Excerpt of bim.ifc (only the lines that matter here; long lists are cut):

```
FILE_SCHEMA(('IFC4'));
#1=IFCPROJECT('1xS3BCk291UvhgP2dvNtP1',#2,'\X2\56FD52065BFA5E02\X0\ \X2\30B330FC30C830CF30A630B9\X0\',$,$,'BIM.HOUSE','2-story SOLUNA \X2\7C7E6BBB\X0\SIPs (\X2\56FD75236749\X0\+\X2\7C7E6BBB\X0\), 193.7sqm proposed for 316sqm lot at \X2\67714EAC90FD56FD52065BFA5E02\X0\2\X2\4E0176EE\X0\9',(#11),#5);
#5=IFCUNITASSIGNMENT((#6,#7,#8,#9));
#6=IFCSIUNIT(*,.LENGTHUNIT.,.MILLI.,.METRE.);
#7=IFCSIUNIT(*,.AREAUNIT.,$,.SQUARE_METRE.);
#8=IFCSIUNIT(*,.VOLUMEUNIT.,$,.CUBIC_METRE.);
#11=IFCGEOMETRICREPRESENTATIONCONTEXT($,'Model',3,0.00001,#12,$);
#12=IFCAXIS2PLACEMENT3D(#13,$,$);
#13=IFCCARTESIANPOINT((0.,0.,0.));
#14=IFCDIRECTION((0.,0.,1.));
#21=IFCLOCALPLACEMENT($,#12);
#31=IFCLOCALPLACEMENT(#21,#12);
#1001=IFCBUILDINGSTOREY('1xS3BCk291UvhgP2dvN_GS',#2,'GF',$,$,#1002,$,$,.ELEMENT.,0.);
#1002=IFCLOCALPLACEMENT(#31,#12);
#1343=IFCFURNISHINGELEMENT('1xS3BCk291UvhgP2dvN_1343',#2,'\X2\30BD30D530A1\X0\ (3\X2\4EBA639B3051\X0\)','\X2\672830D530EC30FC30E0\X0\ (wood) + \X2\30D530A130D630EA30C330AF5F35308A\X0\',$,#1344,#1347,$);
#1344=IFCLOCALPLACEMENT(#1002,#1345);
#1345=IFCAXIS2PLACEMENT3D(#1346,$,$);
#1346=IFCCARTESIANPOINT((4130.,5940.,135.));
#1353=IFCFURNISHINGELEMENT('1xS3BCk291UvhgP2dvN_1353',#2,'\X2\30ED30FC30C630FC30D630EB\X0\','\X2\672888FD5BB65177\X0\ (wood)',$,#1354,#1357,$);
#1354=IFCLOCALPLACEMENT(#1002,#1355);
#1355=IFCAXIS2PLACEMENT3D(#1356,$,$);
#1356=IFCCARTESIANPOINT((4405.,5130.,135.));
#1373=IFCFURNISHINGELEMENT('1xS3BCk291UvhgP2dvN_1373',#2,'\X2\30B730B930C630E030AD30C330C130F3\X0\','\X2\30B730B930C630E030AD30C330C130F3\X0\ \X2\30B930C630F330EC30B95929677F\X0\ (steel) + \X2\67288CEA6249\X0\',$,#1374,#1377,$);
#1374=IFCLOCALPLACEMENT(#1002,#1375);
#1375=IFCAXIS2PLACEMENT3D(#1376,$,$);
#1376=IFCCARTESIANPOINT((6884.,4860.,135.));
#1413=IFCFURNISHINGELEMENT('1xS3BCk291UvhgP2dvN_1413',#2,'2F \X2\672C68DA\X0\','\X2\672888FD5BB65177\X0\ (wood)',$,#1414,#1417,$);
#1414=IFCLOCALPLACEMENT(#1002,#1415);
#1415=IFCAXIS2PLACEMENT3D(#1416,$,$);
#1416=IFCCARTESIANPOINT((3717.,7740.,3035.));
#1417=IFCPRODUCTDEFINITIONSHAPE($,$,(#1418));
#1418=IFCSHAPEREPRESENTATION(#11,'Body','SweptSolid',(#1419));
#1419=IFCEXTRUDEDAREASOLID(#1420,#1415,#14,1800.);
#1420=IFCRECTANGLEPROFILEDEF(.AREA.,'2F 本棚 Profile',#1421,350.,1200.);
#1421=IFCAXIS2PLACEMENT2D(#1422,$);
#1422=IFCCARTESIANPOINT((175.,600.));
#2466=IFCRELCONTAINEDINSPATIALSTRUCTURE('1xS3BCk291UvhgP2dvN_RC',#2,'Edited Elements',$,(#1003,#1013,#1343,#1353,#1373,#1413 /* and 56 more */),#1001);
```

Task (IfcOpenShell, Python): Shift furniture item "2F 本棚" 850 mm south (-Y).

```python
import ifcopenshell
import ifcopenshell.api.geometry
import ifcopenshell.util.placement

model = ifcopenshell.open("bim.ifc")

item = model.by_guid("1xS3BCk291UvhgP2dvN_1413")
matrix = ifcopenshell.util.placement.get_local_placement(item.ObjectPlacement)
matrix[1, 3] -= 850.0
ifcopenshell.api.geometry.edit_object_placement(model, product=item, matrix=matrix, is_si=False)

print(ifcopenshell.util.placement.get_local_placement(item.ObjectPlacement).round(3) + 0.0)

model.write("bim_v2.ifc")
```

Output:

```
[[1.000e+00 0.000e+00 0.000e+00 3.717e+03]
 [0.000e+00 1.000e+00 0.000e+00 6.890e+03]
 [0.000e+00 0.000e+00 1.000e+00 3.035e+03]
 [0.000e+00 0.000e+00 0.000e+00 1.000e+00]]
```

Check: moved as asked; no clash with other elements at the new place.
